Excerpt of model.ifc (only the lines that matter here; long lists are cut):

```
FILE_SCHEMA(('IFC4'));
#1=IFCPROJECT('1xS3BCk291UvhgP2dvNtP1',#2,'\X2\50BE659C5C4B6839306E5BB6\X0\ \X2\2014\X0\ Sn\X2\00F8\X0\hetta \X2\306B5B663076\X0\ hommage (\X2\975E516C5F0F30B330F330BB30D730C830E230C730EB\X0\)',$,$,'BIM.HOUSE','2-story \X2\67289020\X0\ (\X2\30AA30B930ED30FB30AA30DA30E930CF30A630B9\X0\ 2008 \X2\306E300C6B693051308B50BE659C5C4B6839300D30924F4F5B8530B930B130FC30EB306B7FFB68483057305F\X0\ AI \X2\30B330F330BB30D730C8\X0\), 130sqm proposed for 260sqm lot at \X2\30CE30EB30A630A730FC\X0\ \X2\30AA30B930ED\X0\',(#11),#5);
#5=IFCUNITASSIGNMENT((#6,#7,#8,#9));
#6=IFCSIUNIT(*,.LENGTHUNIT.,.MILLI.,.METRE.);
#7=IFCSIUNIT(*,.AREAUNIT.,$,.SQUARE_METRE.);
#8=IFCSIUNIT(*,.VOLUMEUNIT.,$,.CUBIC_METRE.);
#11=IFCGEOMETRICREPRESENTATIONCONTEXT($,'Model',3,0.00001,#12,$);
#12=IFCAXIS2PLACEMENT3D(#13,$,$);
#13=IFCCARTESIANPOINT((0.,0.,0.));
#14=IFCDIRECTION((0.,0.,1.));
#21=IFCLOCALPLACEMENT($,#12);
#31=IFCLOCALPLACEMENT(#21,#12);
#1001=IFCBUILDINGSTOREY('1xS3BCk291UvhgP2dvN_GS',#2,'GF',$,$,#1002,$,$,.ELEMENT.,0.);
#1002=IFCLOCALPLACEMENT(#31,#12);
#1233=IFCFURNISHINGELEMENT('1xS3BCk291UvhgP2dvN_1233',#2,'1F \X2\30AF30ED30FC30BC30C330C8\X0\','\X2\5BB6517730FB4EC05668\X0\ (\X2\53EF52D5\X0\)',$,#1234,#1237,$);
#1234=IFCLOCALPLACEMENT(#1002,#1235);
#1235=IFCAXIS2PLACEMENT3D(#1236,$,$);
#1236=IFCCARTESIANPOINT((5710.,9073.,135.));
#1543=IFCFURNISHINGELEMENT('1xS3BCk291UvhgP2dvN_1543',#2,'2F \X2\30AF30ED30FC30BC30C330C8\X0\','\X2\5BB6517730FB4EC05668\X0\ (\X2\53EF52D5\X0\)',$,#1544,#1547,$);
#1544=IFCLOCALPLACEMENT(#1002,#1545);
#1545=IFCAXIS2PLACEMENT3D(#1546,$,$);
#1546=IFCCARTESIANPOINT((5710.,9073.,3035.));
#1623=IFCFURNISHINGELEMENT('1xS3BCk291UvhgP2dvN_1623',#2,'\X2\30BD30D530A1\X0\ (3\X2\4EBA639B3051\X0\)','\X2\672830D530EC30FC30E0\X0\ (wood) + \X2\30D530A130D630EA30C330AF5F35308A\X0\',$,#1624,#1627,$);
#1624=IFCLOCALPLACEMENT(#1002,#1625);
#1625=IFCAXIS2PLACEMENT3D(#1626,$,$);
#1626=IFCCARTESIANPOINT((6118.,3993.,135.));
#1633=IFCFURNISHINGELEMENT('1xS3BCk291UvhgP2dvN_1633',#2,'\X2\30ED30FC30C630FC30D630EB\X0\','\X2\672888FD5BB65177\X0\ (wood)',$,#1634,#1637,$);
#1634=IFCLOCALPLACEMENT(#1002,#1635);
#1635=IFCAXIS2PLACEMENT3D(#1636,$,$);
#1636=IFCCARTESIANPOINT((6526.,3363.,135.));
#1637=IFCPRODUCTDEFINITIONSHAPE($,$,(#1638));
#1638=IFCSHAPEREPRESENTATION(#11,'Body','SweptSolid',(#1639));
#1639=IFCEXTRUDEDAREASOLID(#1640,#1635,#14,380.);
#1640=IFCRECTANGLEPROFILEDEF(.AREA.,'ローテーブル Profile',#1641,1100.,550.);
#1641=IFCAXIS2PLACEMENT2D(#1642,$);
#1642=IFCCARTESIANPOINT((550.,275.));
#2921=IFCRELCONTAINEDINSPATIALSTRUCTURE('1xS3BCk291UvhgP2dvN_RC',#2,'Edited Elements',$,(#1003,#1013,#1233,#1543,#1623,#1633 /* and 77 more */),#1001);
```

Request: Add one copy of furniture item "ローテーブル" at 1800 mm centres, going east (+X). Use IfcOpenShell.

```python
import numpy as np
import ifcopenshell
import ifcopenshell.api.geometry
import ifcopenshell.api.root
import ifcopenshell.util.element
import ifcopenshell.util.placement
import ifcopenshell.util.unit

model = ifcopenshell.open("model.ifc")
unit_scale = ifcopenshell.util.unit.calculate_unit_scale(model)


def reuse_history(source, copy):
    """copy_class also copies each property set's owner history, people and application; keep the originals."""
    for rel in copy.IsDefinedBy:
        if rel.is_a("IfcRelDefinesByProperties") and (history := rel.RelatingPropertyDefinition.OwnerHistory):
            rel.RelatingPropertyDefinition.OwnerHistory = source.OwnerHistory
            ifcopenshell.util.element.remove_deep2(model, history)


source = model.by_guid("1xS3BCk291UvhgP2dvN_1633")
base = ifcopenshell.util.placement.get_local_placement(source.ObjectPlacement)
step = np.array([1.0, 0.0, 0.0]) * 1.8 / unit_scale

for i in range(1, 2):
    copy = ifcopenshell.api.root.copy_class(model, product=source)
    copy.Representation = ifcopenshell.util.element.copy_deep(
        model, source.Representation, exclude=["IfcGeometricRepresentationContext", "IfcRepresentationMap"]
    )
    reuse_history(source, copy)
    matrix = base.copy()
    matrix[:3, 3] += i * step
    print("added at", matrix[:3, 3].round(3) + 0.0)
    ifcopenshell.api.geometry.edit_object_placement(model, product=copy, matrix=matrix, is_si=False)

model.write("model_v2.ifc")
```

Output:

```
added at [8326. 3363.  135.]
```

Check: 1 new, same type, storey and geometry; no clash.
